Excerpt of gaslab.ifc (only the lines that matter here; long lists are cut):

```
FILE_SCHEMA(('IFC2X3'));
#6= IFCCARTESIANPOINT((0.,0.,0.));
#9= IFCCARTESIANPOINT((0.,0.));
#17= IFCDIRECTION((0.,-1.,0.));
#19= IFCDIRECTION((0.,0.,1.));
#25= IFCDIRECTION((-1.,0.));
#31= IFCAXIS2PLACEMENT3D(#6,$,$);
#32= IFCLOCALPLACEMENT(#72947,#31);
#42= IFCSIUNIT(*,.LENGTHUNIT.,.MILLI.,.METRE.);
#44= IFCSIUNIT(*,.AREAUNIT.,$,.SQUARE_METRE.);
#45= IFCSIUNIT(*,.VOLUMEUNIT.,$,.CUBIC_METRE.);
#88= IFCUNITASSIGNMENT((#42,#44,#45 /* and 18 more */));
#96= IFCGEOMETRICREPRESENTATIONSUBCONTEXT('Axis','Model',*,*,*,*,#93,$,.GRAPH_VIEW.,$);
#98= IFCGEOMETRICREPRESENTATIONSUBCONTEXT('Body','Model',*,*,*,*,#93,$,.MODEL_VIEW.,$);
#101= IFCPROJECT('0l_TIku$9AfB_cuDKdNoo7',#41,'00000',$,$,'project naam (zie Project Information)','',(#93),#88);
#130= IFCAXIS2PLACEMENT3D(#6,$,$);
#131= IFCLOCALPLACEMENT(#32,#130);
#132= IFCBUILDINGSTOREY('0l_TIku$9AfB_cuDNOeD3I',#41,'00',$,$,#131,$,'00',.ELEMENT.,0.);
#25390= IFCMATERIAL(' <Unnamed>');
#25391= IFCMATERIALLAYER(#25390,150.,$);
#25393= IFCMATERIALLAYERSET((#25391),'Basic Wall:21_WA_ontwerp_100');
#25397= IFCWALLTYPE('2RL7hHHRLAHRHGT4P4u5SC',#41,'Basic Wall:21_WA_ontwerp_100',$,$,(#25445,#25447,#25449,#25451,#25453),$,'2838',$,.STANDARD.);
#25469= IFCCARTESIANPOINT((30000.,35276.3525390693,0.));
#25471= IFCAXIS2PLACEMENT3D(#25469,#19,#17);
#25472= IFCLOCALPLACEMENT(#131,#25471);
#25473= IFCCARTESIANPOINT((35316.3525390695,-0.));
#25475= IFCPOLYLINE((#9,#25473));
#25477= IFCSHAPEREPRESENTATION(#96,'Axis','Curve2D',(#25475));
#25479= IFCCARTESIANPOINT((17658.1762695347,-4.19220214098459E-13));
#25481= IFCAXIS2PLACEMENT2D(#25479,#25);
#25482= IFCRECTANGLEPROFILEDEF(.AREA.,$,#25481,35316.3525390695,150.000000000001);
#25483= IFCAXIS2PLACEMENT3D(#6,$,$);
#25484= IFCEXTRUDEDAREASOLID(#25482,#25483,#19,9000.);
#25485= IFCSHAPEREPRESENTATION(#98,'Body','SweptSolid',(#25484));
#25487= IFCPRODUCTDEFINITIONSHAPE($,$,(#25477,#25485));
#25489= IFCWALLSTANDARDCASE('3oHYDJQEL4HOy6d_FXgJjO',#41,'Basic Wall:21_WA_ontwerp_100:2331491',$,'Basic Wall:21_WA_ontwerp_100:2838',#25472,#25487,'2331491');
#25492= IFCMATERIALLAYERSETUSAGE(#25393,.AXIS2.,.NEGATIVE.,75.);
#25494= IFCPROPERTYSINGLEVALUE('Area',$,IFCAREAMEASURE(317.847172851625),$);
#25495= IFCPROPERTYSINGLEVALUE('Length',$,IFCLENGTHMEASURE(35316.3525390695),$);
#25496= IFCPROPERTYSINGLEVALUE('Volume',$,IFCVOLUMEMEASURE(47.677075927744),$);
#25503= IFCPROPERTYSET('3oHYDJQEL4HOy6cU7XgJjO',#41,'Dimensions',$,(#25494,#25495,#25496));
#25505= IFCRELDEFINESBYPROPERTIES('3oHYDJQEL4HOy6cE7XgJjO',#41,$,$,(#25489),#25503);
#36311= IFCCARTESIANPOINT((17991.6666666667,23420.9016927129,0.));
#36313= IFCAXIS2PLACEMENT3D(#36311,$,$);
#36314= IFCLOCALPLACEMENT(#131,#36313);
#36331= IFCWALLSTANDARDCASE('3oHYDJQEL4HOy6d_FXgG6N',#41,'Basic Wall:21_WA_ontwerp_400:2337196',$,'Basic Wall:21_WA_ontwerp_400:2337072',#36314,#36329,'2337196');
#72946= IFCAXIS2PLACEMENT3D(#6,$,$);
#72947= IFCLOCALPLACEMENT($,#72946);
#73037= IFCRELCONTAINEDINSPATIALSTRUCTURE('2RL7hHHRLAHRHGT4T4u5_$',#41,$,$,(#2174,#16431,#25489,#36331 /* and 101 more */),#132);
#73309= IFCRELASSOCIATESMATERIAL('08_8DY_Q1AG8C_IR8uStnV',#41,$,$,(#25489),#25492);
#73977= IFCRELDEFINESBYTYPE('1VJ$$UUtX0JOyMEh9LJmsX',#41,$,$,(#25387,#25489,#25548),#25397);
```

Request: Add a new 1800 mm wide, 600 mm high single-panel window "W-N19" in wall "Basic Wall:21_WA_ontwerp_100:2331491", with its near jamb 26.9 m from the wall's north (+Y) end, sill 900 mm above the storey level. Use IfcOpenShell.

```python
import numpy as np
import ifcopenshell
import ifcopenshell.api.feature
import ifcopenshell.api.geometry
import ifcopenshell.api.pset
import ifcopenshell.api.root
import ifcopenshell.api.spatial
import ifcopenshell.api.type
import ifcopenshell.geom
import ifcopenshell.util.element
import ifcopenshell.util.placement
import ifcopenshell.util.representation
import ifcopenshell.util.shape
import ifcopenshell.util.unit

model = ifcopenshell.open("gaslab.ifc")
unit_scale = ifcopenshell.util.unit.calculate_unit_scale(model)
area_scale = ifcopenshell.util.unit.calculate_unit_scale(model, "AREAUNIT")
volume_scale = ifcopenshell.util.unit.calculate_unit_scale(model, "VOLUMEUNIT")
settings = ifcopenshell.geom.settings()


def volume(element):
    """Net volume in cubic metres, openings subtracted."""
    shape = ifcopenshell.geom.create_shape(settings, element)
    return ifcopenshell.util.shape.get_volume(shape.geometry)


wall = model.by_guid("3oHYDJQEL4HOy6d_FXgJjO")
storey = ifcopenshell.util.element.get_container(wall, ifc_class="IfcBuildingStorey")
context = ifcopenshell.util.representation.get_context(model, "Model", "Body", "MODEL_VIEW")
before = volume(wall)

width, height, from_end, sill = 1.8, 0.6, 26.9, 0.9  # metres

# The wall runs along its own X axis, and the end named is its -X end.
wall_shape = ifcopenshell.geom.create_shape(settings, wall)
x, y, z = ifcopenshell.util.shape.get_vertices(wall_shape.geometry).T
start = x.min() + from_end
face, thickness = float(y.min()), float(y.max() - y.min())
wall_matrix = ifcopenshell.util.placement.get_local_placement(wall.ObjectPlacement)
level = ifcopenshell.util.placement.get_local_placement(storey.ObjectPlacement)[2, 3]


def in_wall(x, y):
    """Placement at x, y metres in the wall's axes, at sill height."""
    matrix = wall_matrix.copy()
    matrix[:, 3] = wall_matrix @ np.array([x / unit_scale, y / unit_scale, 0.0, 1.0])
    matrix[2, 3] = level + sill / unit_scale
    return matrix


# Opening: a box that overshoots both wall faces by 50 mm.
opening = ifcopenshell.api.root.create_entity(model, ifc_class="IfcOpeningElement")
box = ifcopenshell.api.geometry.add_wall_representation(
    model, context=context, length=width, height=height, thickness=thickness + 0.1
)
ifcopenshell.api.geometry.assign_representation(model, product=opening, representation=box)
ifcopenshell.api.geometry.edit_object_placement(model, product=opening, matrix=in_wall(start, face - 0.05), is_si=False)
ifcopenshell.api.feature.add_feature(model, feature=opening, element=wall)

window = ifcopenshell.api.root.create_entity(model, ifc_class="IfcWindow", name="W-N19")
window.OverallWidth, window.OverallHeight = width / unit_scale, height / unit_scale
body = ifcopenshell.api.geometry.add_window_representation(
    model,
    context=context,
    overall_width=window.OverallWidth,
    overall_height=window.OverallHeight,
    partition_type="SINGLE_PANEL",
)
ifcopenshell.api.geometry.assign_representation(model, product=window, representation=body)
ifcopenshell.api.spatial.assign_container(model, products=[window], relating_structure=storey)
fills = ifcopenshell.api.feature.add_filling(model, opening=opening, element=window)
fills.OwnerHistory = window.OwnerHistory  # required in IFC2X3

# IFC2X3 keeps the operation on the window style.
style = ifcopenshell.api.root.create_entity(model, ifc_class="IfcWindowStyle", name="W-N19")
style.OperationType, style.ConstructionType = "SINGLE_PANEL", "NOTDEFINED"
style.ParameterTakesPrecedence = style.Sizeable = False
ifcopenshell.api.type.assign_type(model, related_objects=[window], relating_type=style)

# Centre the window in the wall's thickness.
ifcopenshell.api.geometry.edit_object_placement(model, product=window, matrix=in_wall(start, face), is_si=False)
window_shape = ifcopenshell.geom.create_shape(settings, window)
depth = ifcopenshell.util.shape.get_vertices(window_shape.geometry)[:, 1]
offset = face + thickness / 2 - (depth.min() + depth.max()) / 2
ifcopenshell.api.geometry.edit_object_placement(model, product=window, matrix=in_wall(start, offset), is_si=False)

after = volume(wall)

# Update the wall's stored quantities.
pset = model.by_id(ifcopenshell.util.element.get_pset(wall, "Dimensions", should_inherit=False)["id"])
ifcopenshell.api.pset.edit_pset(model, pset=pset, properties={
    "Area": model.create_entity("IfcAreaMeasure", after / thickness / area_scale),
    "Volume": model.create_entity("IfcVolumeMeasure", after / volume_scale),
})

print(f"wall volume {before:.3f} -> {after:.3f} m3")

model.write("gaslab_rev.ifc")
```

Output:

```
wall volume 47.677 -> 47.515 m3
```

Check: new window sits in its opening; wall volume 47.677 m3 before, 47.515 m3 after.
